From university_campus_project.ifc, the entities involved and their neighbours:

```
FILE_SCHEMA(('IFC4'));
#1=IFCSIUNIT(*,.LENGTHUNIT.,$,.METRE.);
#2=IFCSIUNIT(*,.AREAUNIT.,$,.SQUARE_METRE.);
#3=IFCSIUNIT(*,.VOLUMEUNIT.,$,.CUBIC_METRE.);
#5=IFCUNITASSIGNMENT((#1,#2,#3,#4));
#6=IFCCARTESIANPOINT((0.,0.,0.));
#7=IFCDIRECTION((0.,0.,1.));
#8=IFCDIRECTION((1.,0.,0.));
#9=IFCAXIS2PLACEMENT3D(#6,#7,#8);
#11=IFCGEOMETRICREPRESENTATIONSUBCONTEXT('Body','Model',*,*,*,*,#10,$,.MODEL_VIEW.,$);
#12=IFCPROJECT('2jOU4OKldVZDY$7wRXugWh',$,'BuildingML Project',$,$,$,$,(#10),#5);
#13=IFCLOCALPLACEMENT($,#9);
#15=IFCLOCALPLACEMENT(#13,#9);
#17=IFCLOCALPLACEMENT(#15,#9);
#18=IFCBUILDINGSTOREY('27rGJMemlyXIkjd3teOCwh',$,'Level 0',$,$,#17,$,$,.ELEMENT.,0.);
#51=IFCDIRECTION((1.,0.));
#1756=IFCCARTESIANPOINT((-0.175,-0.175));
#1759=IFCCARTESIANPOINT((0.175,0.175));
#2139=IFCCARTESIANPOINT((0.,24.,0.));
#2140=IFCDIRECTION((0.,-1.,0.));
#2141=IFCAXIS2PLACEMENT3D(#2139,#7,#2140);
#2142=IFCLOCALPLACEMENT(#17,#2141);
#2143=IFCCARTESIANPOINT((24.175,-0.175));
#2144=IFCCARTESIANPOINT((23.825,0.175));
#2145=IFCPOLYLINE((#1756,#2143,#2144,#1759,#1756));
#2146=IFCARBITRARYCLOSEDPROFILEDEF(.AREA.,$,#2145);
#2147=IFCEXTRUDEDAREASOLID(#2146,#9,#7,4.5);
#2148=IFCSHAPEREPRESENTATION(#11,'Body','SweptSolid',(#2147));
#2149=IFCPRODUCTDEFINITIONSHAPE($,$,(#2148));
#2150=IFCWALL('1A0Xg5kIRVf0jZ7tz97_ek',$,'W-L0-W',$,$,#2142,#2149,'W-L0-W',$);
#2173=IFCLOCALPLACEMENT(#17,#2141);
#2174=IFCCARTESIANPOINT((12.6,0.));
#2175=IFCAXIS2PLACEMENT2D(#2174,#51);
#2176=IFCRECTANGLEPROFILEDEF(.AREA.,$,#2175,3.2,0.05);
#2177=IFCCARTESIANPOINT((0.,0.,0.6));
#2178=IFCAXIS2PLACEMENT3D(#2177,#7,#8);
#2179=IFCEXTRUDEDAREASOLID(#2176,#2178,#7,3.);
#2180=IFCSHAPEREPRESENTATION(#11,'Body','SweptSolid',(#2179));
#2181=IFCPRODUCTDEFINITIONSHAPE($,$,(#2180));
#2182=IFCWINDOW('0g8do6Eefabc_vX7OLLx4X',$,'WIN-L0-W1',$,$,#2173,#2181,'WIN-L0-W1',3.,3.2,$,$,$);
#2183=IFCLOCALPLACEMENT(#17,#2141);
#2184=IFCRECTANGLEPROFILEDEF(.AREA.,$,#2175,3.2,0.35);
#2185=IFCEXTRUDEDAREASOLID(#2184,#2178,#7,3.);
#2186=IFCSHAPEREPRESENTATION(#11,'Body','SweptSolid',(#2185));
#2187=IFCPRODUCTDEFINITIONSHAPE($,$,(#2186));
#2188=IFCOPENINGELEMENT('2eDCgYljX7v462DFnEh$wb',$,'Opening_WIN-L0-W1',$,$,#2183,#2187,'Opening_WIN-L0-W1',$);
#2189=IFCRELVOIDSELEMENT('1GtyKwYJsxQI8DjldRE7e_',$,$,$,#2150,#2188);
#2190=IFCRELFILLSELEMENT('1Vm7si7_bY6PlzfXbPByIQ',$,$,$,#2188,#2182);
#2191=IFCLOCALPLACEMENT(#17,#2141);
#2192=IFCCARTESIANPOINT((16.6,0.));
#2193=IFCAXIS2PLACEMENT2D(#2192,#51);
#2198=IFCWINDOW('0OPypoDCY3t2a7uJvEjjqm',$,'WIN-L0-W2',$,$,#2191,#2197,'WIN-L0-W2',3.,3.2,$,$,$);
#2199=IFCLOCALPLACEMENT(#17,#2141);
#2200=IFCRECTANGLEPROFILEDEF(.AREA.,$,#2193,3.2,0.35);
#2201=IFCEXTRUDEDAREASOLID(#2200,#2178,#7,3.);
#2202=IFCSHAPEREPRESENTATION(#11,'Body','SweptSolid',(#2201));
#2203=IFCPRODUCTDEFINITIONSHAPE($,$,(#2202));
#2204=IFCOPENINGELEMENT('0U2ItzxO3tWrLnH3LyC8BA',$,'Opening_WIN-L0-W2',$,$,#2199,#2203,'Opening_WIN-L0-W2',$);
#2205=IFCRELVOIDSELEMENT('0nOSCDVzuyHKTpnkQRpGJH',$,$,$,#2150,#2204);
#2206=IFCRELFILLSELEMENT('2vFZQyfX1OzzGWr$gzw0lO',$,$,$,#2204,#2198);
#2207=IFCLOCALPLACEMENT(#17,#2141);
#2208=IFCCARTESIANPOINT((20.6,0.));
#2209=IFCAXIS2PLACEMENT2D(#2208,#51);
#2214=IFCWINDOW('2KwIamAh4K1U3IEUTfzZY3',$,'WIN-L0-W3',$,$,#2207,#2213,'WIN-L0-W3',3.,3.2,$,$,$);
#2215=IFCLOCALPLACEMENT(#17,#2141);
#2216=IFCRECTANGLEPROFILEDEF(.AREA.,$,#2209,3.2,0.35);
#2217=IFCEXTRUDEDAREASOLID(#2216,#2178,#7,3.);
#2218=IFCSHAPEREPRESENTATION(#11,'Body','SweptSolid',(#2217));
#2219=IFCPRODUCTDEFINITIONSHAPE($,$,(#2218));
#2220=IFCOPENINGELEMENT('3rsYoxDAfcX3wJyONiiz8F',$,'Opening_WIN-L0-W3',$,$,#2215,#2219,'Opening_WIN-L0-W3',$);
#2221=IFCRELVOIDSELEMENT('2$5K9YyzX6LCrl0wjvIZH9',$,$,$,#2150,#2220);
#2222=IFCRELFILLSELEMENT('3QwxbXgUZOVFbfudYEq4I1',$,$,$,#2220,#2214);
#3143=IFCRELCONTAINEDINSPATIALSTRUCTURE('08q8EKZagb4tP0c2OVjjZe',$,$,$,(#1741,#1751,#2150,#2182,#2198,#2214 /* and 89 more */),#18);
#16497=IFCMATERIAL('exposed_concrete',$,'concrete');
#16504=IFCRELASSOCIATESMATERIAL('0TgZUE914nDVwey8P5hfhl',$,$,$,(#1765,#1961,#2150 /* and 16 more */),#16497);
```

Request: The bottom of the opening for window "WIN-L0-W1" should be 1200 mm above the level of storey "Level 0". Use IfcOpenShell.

```python
import numpy as np
import ifcopenshell
import ifcopenshell.api.geometry
import ifcopenshell.geom
import ifcopenshell.util.element
import ifcopenshell.util.placement
import ifcopenshell.util.shape
import ifcopenshell.util.unit

model = ifcopenshell.open("university_campus_project.ifc")
unit_scale = ifcopenshell.util.unit.calculate_unit_scale(model)

window = model.by_guid("0g8do6Eefabc_vX7OLLx4X")
opening = window.FillsVoids[0].RelatingOpeningElement
storey = ifcopenshell.util.element.get_container(window, ifc_class="IfcBuildingStorey")
level = ifcopenshell.util.placement.get_local_placement(storey.ObjectPlacement)[2, 3]

# The opening's origin need not be at the sill, so measure its lowest point.
shape = ifcopenshell.geom.create_shape(ifcopenshell.geom.settings(), opening)
bottom = ifcopenshell.util.shape.get_shape_bottom_elevation(shape, shape.geometry) / unit_scale
dz = level + 1.2 / unit_scale - bottom

shift = np.array([0.0, 0.0, dz])
# The window is not placed relative to its opening, so move both.
for product in (opening, window):
    matrix = ifcopenshell.util.placement.get_local_placement(product.ObjectPlacement)
    matrix[:3, 3] += shift
    ifcopenshell.api.geometry.edit_object_placement(model, product=product, matrix=matrix, is_si=False)

print(f"moved by {dz * unit_scale:+.3f} m")

model.write("university_campus_project_edited.ifc")
```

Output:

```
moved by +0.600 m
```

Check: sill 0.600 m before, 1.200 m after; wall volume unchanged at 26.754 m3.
